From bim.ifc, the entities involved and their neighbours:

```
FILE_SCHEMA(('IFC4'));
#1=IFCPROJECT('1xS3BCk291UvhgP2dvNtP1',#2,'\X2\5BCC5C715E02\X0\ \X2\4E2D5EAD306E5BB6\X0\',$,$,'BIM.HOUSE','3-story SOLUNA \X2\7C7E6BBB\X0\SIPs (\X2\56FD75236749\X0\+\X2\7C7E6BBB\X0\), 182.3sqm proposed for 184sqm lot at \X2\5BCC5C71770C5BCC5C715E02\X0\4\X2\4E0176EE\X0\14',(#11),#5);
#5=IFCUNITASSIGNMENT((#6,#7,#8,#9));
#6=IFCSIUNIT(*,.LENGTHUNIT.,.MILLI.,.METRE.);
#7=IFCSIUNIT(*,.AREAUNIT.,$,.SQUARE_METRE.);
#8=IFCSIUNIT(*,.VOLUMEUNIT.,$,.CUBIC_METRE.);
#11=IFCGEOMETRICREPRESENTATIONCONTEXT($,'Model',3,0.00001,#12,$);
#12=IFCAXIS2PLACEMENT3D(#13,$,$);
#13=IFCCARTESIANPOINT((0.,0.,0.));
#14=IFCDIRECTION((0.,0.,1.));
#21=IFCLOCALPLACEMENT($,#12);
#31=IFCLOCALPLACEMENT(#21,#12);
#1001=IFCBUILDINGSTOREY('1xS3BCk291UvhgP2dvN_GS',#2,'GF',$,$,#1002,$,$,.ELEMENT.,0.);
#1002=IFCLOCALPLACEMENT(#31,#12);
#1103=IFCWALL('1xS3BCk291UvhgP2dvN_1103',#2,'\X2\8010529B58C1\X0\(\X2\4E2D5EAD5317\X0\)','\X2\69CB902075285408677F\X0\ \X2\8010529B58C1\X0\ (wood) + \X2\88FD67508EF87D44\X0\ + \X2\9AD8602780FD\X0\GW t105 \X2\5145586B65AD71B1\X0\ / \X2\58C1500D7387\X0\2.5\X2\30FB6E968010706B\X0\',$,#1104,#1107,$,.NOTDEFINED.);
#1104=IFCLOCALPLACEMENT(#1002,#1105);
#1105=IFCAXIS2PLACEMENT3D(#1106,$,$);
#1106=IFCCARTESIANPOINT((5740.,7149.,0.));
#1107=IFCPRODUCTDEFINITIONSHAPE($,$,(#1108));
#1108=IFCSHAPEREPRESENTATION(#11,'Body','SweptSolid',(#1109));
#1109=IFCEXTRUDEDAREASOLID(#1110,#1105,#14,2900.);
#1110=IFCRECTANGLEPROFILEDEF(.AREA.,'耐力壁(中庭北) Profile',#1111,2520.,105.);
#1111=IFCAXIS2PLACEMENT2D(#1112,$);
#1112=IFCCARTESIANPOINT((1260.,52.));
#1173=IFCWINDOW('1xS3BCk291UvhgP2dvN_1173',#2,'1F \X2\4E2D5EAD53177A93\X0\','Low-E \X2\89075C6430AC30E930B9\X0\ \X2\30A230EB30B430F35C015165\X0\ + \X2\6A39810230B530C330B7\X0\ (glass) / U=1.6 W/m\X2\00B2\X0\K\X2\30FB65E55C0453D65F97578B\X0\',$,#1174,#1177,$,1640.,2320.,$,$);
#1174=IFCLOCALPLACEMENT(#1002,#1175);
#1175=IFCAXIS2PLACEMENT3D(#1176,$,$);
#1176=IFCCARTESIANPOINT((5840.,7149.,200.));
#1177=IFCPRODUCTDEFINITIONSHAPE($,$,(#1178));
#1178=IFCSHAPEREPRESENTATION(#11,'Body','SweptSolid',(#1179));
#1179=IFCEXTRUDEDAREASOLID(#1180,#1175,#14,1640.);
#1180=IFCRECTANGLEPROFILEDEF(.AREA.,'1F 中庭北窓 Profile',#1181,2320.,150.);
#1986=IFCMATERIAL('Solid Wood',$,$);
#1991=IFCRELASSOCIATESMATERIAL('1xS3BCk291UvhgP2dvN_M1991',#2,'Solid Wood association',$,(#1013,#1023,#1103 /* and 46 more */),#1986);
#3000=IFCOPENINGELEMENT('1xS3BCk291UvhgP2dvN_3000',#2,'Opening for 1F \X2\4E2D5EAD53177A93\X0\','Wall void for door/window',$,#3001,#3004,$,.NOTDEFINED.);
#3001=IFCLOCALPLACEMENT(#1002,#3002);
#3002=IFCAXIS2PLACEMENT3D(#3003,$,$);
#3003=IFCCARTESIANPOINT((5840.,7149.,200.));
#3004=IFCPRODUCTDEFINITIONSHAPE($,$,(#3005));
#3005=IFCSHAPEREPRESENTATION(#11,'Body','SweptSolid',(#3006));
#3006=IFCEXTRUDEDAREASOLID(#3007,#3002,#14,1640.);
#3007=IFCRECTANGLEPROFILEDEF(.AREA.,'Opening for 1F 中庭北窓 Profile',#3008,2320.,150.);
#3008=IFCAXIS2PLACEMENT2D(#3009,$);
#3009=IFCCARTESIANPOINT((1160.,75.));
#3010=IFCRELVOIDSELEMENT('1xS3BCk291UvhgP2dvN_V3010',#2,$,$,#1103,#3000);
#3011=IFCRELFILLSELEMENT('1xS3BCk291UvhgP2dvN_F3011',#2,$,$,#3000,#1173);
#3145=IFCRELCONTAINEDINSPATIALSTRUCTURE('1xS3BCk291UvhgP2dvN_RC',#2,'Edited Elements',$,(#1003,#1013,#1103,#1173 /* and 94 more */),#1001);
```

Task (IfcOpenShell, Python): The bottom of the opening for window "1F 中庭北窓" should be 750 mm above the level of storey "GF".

```python
import numpy as np
import ifcopenshell
import ifcopenshell.api.geometry
import ifcopenshell.geom
import ifcopenshell.util.element
import ifcopenshell.util.placement
import ifcopenshell.util.shape
import ifcopenshell.util.unit

model = ifcopenshell.open("bim.ifc")
unit_scale = ifcopenshell.util.unit.calculate_unit_scale(model)

window = model.by_id(1173)
opening = window.FillsVoids[0].RelatingOpeningElement
storey = ifcopenshell.util.element.get_container(window, ifc_class="IfcBuildingStorey")
level = ifcopenshell.util.placement.get_local_placement(storey.ObjectPlacement)[2, 3]

# The opening's origin need not be at the sill, so measure its lowest point.
shape = ifcopenshell.geom.create_shape(ifcopenshell.geom.settings(), opening)
bottom = ifcopenshell.util.shape.get_shape_bottom_elevation(shape, shape.geometry) / unit_scale
dz = level + 750.0 - bottom

shift = np.array([0.0, 0.0, dz])
# The window is not placed relative to its opening, so move both.
for product in (opening, window):
    matrix = ifcopenshell.util.placement.get_local_placement(product.ObjectPlacement)
    matrix[:3, 3] += shift
    ifcopenshell.api.geometry.edit_object_placement(model, product=product, matrix=matrix, is_si=False)

print(f"moved by {dz * unit_scale:+.3f} m")

model.write("bim-out.ifc")
```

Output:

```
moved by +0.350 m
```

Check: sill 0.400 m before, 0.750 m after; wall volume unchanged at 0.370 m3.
